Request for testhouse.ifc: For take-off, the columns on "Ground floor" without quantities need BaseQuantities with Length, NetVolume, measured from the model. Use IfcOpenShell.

First a look at what the model holds.

```python
import ifcopenshell
import ifcopenshell.util.element
import ifcopenshell.util.unit

model = ifcopenshell.open("testhouse.ifc")
print(model.schema)
for unit_type in ("LENGTHUNIT", "AREAUNIT", "VOLUMEUNIT"):
    print(unit_type, ifcopenshell.util.unit.calculate_unit_scale(model, unit_type))
storey = next(s for s in model.by_type("IfcBuildingStorey") if s.Name == "Ground floor")
columns = [e for e in ifcopenshell.util.element.get_decomposition(storey) if e.is_a("IfcColumn")]
for e in sorted(columns, key=lambda e: e.id()):
    print(e.id(), e.is_a(), e.Name, list(ifcopenshell.util.element.get_psets(e, qtos_only=True)), sep=" | ")
```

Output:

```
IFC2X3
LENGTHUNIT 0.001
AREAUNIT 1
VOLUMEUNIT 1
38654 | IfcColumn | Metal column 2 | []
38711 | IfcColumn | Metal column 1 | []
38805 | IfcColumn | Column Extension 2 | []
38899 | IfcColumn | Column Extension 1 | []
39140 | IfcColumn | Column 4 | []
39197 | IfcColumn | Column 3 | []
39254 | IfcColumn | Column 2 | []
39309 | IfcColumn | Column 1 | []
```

```python
import ifcopenshell
import ifcopenshell.api.pset
import ifcopenshell.geom
import ifcopenshell.util.element
import ifcopenshell.util.shape
import ifcopenshell.util.unit

model = ifcopenshell.open("testhouse.ifc")
unit_scale = ifcopenshell.util.unit.calculate_unit_scale(model)
volume_scale = ifcopenshell.util.unit.calculate_unit_scale(model, "VOLUMEUNIT")
settings = ifcopenshell.geom.settings()

storey = next(s for s in model.by_type("IfcBuildingStorey") if s.Name == "Ground floor")
columns = [e for e in ifcopenshell.util.element.get_decomposition(storey) if e.is_a("IfcColumn")]

for e in sorted(columns, key=lambda e: e.id()):
    if ifcopenshell.util.element.get_psets(e, qtos_only=True, should_inherit=False):
        continue
    # Geometry comes back in metres, in the element's own axes.
    shape = ifcopenshell.geom.create_shape(settings, e)
    values = {
        "Length": ifcopenshell.util.shape.get_z(shape.geometry) / unit_scale,
        "NetVolume": ifcopenshell.util.shape.get_volume(shape.geometry) / volume_scale,
    }
    qto = ifcopenshell.api.pset.add_qto(model, product=e, name="BaseQuantities")
    ifcopenshell.api.pset.edit_qto(model, qto=qto, properties=values)
    print(e.id(), {k: round(v, 3) for k, v in values.items()})

model.write("testhouse_rev.ifc")
```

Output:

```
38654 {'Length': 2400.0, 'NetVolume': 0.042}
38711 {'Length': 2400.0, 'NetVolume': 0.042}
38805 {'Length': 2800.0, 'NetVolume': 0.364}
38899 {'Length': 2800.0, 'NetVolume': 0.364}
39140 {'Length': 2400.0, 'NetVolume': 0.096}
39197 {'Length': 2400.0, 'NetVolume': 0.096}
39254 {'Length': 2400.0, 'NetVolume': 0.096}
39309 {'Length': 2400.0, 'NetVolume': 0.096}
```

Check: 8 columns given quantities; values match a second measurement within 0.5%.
